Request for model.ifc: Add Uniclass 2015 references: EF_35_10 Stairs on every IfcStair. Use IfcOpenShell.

First a look at what the model holds.

```python
import ifcopenshell

model = ifcopenshell.open("model.ifc")
print(model.schema)
print("classifications:", [c.Name for c in model.by_type("IfcClassification")])
for ifc_class in ("IfcDoor", "IfcRoof", "IfcStair", "IfcWall", "IfcWindow"):
    print(ifc_class, len(model.by_type(ifc_class)))
```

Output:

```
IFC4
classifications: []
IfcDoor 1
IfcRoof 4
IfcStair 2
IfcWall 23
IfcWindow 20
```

```python
import ifcopenshell
import ifcopenshell.api.classification

model = ifcopenshell.open("model.ifc")

system = ifcopenshell.api.classification.add_classification(model, classification="Uniclass 2015")

codes = {
    "IfcStair": ("EF_35_10", "Stairs"),
}
for ifc_class, (code, name) in codes.items():
    products = model.by_type(ifc_class)
    ifcopenshell.api.classification.add_reference(
        model, products=products, classification=system, identification=code, name=name
    )
    print(code, len(products))

model.write("model_v2.ifc")
```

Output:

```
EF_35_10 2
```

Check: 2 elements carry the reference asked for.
